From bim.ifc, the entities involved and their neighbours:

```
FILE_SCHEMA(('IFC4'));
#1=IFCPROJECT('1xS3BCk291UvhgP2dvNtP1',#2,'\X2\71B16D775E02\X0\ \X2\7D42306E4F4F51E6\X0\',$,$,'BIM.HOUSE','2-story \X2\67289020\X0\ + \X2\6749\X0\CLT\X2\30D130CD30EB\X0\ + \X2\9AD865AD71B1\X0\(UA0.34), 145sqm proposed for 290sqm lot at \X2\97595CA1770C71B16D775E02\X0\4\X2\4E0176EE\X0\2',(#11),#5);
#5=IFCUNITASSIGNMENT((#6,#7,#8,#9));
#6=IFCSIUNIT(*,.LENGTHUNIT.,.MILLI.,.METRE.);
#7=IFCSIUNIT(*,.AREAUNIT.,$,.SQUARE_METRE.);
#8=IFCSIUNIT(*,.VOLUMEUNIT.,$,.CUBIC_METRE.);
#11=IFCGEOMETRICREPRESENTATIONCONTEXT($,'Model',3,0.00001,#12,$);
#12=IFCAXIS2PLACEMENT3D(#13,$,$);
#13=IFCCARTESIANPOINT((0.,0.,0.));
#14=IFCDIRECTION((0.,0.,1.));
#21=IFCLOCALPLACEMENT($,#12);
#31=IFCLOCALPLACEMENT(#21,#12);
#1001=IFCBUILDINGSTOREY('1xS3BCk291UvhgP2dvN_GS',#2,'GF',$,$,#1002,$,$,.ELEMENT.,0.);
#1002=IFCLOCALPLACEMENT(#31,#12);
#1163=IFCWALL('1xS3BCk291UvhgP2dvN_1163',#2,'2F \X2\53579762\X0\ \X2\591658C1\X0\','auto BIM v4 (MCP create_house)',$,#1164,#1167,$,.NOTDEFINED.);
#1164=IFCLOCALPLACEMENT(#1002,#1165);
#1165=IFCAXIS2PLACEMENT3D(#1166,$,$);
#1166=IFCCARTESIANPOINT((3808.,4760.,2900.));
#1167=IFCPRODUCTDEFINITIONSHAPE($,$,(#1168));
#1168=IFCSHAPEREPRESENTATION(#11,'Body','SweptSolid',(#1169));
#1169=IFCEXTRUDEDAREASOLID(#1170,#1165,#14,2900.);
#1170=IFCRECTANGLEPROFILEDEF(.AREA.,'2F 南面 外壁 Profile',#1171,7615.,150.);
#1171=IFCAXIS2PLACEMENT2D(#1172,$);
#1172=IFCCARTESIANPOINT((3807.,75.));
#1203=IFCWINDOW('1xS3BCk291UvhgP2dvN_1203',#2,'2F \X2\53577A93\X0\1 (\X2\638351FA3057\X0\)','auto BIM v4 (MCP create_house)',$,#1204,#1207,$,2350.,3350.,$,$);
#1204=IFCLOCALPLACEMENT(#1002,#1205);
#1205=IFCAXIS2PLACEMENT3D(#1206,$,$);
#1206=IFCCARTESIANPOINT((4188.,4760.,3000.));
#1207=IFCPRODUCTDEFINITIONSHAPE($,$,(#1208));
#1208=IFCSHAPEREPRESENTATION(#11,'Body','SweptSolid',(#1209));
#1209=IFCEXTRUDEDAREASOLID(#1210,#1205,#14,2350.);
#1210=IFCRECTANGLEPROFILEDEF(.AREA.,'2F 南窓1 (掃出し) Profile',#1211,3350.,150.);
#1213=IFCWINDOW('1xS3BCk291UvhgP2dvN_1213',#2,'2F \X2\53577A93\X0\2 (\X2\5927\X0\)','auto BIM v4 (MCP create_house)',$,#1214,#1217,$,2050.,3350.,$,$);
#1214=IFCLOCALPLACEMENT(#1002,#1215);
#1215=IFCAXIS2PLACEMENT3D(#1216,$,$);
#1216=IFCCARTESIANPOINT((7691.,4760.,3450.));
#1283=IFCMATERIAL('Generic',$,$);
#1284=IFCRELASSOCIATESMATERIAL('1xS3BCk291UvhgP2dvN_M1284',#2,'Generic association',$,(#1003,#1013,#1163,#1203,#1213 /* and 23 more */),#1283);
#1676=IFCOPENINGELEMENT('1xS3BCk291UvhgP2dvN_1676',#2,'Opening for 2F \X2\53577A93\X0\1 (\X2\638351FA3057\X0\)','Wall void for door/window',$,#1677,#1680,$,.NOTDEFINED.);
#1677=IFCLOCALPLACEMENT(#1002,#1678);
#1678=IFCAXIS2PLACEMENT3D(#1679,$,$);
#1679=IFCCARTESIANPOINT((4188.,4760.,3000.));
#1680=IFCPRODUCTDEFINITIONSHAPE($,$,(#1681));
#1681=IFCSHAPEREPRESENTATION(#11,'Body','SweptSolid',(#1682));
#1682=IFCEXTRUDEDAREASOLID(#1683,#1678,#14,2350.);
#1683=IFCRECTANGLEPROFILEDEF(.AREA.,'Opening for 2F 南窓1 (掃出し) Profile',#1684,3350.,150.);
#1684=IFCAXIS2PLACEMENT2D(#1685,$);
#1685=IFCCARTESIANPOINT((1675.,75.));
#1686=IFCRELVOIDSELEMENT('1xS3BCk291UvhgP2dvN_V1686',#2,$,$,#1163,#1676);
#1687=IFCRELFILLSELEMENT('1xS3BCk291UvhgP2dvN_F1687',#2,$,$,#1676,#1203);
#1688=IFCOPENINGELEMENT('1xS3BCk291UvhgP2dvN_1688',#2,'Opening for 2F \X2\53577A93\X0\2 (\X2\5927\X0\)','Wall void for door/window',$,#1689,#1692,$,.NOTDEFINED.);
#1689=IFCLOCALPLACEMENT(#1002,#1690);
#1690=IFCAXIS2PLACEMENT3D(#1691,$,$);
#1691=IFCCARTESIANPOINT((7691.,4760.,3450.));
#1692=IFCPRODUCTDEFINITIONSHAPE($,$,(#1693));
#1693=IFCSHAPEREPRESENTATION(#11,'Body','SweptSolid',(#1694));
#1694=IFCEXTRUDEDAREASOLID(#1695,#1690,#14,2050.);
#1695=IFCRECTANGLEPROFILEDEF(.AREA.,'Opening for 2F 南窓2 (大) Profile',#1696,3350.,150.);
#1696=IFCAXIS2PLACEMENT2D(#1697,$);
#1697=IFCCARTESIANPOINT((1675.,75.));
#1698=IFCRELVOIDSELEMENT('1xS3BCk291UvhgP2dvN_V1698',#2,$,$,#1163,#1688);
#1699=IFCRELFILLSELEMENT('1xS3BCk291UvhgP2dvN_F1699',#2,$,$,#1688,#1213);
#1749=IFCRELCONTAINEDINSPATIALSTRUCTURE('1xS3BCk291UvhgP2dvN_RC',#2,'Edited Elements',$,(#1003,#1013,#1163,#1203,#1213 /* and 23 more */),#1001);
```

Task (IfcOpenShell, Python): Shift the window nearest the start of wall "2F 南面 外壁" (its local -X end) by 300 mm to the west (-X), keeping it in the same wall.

```python
import ifcopenshell
import ifcopenshell.api.geometry
import ifcopenshell.util.placement
import ifcopenshell.util.unit

model = ifcopenshell.open("bim.ifc")
unit_scale = ifcopenshell.util.unit.calculate_unit_scale(model)

window = model.by_guid("1xS3BCk291UvhgP2dvN_1203")
opening = window.FillsVoids[0].RelatingOpeningElement
wall = opening.VoidsElements[0].RelatingBuildingElement

wall_matrix = ifcopenshell.util.placement.get_local_placement(wall.ObjectPlacement)
shift = wall_matrix[:3, 0] * -0.3 / unit_scale
before = ifcopenshell.util.placement.get_local_placement(window.ObjectPlacement)[:3, 3].copy()

# The window is not placed relative to its opening, so move both.
for product in (opening, window):
    matrix = ifcopenshell.util.placement.get_local_placement(product.ObjectPlacement)
    matrix[:3, 3] += shift
    ifcopenshell.api.geometry.edit_object_placement(model, product=product, matrix=matrix, is_si=False)

after = ifcopenshell.util.placement.get_local_placement(window.ObjectPlacement)[:3, 3]
print("window moved by", (after - before).round(3) + 0.0)

model.write("bim_updated.ifc")
```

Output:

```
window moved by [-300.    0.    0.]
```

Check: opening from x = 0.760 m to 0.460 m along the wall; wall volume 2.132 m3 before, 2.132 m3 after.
